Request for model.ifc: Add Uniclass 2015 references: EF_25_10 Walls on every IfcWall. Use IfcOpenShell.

First a look at what the model holds.

```python
import ifcopenshell

model = ifcopenshell.open("model.ifc")
print(model.schema)
print("classifications:", [c.Name for c in model.by_type("IfcClassification")])
for ifc_class in ("IfcDoor", "IfcRoof", "IfcStair", "IfcWall", "IfcWindow"):
    print(ifc_class, len(model.by_type(ifc_class)))
```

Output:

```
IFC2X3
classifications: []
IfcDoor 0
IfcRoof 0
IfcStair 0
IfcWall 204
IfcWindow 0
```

```python
import ifcopenshell
import ifcopenshell.api.classification

model = ifcopenshell.open("model.ifc")

# IFC2X3 requires Source and Edition and has no link from the project to the system.
system = model.create_entity("IfcClassification", Source="NBS", Edition="2015", Name="Uniclass 2015")

codes = {
    "IfcWall": ("EF_25_10", "Walls"),
}
for ifc_class, (code, name) in codes.items():
    products = model.by_type(ifc_class)
    ifcopenshell.api.classification.add_reference(
        model, products=products, classification=system, identification=code, name=name
    )
    print(code, len(products))

model.write("model_updated.ifc")
```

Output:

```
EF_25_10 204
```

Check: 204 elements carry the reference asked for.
